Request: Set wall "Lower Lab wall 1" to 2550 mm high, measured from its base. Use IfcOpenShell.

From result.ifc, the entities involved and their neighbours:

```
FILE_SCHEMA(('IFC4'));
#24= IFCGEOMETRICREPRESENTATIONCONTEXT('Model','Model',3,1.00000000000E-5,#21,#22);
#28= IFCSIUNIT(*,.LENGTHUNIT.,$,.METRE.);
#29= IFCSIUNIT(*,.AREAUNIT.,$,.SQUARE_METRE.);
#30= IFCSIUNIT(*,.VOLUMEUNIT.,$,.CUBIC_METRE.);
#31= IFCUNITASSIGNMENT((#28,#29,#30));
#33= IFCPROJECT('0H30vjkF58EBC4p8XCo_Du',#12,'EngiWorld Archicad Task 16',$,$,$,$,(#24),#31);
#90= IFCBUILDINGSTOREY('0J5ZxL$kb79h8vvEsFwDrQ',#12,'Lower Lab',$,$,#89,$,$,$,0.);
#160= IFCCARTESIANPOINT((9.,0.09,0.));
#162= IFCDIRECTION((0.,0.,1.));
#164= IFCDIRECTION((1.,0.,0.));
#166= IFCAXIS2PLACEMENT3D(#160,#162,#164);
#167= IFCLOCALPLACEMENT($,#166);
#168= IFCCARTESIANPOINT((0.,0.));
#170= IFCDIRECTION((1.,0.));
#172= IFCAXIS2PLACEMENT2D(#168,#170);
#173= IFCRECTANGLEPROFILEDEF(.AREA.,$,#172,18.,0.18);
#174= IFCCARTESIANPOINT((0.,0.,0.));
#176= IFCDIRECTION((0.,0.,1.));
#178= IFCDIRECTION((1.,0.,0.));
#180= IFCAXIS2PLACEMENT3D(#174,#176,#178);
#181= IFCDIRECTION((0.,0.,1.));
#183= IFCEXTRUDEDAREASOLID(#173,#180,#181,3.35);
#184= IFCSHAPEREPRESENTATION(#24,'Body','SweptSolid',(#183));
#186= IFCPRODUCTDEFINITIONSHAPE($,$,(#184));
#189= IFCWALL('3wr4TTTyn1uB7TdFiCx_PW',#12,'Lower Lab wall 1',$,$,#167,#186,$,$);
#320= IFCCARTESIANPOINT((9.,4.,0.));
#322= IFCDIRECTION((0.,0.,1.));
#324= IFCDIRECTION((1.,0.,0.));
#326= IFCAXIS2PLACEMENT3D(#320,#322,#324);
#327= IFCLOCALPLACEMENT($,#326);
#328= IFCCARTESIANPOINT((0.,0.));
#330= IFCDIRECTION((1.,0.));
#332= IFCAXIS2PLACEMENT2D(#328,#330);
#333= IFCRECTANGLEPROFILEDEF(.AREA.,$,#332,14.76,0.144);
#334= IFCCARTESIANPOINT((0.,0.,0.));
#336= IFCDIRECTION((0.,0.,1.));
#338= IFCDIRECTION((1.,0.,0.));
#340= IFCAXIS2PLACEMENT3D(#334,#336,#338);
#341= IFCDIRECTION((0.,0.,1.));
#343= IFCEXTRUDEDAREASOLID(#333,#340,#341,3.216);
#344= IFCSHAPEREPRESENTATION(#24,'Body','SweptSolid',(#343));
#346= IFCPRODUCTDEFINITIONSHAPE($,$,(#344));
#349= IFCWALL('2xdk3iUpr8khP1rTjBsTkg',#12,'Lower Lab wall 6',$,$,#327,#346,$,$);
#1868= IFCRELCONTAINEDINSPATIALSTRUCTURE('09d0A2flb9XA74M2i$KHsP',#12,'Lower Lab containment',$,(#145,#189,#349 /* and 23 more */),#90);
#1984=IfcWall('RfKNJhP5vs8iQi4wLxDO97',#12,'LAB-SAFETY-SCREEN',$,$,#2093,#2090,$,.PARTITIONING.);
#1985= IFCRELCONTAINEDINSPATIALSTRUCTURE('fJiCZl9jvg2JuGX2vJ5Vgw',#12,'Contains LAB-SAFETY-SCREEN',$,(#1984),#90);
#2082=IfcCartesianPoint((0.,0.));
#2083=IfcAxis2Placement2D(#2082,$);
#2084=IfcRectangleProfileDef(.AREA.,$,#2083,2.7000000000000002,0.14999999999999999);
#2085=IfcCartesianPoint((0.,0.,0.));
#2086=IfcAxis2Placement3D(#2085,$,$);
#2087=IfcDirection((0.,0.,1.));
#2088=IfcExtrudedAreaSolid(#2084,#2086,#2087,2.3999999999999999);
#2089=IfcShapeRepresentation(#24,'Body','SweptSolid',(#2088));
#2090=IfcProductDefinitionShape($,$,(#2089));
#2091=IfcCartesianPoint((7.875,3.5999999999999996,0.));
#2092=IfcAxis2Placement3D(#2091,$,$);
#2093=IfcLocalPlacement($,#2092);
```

```python
import ifcopenshell
import ifcopenshell.geom
import ifcopenshell.util.shape
import ifcopenshell.util.unit

model = ifcopenshell.open("result.ifc")
unit_scale = ifcopenshell.util.unit.calculate_unit_scale(model)
settings = ifcopenshell.geom.settings()


def volume(element):
    """Net volume in cubic metres, openings subtracted."""
    shape = ifcopenshell.geom.create_shape(settings, element)
    return ifcopenshell.util.shape.get_volume(shape.geometry)


wall = model.by_guid("3wr4TTTyn1uB7TdFiCx_PW")
before = volume(wall)

body = next(r for r in wall.Representation.Representations if r.RepresentationIdentifier == "Body")
solid = body.Items[0]
old_height = solid.Depth
solid.Depth = 2.55 / unit_scale
after = volume(wall)

print(f"height {old_height:g} -> {solid.Depth:g}, volume {before:.3f} -> {after:.3f} m3")

model.write("result_v2.ifc")
```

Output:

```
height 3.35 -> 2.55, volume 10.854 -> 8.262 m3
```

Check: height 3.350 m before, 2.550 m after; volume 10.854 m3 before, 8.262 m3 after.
